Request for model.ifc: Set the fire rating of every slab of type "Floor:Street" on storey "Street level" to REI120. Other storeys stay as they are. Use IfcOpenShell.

First a look at what the model holds.

```python
import ifcopenshell
import ifcopenshell.util.element

model = ifcopenshell.open("model.ifc")
print(model.schema)
storey = next(s for s in model.by_type("IfcBuildingStorey") if s.Name == "Street level")
slabs = [e for e in ifcopenshell.util.element.get_decomposition(storey) if e.is_a("IfcSlab")]
seen = {}
for e in slabs:
    element_type = ifcopenshell.util.element.get_type(e)
    key = (element_type.Name if element_type != e and element_type else None, ifcopenshell.util.element.get_pset(e, "Pset_SlabCommon", "FireRating"))
    seen[key] = seen.get(key, 0) + 1
for (name, value), count in sorted(seen.items(), key=str):
    print(count, "x", name, "|", value)
```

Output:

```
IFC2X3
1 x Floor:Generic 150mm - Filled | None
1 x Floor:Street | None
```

```python
import ifcopenshell
import ifcopenshell.api.pset
import ifcopenshell.util.element

model = ifcopenshell.open("model.ifc")

storey = next(s for s in model.by_type("IfcBuildingStorey") if s.Name == "Street level")
slabs = [e for e in ifcopenshell.util.element.get_decomposition(storey) if e.is_a("IfcSlab")]

count = 0
for e in slabs:
    element_type = ifcopenshell.util.element.get_type(e)
    if element_type in (None, e) or element_type.Name != "Floor:Street":
        continue
    # add_pset returns the element's existing set when there is one.
    pset = ifcopenshell.api.pset.add_pset(model, product=e, name="Pset_SlabCommon")
    ifcopenshell.api.pset.edit_pset(model, pset=pset, properties={"FireRating": "REI120"})
    count += 1

print(count, "slabs updated")

model.write("model_updated.ifc")
```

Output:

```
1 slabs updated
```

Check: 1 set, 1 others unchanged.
